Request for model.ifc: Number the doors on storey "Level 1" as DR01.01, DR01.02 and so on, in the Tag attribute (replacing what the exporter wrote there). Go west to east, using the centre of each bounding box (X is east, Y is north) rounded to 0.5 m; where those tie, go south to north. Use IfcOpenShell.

First a look at what the model holds.

```python
import ifcopenshell
import ifcopenshell.util.element
import ifcopenshell.util.placement

model = ifcopenshell.open("model.ifc")
print(model.schema)
storey = next(s for s in model.by_type("IfcBuildingStorey") if s.Name == "Level 1")
doors = [e for e in ifcopenshell.util.element.get_decomposition(storey) if e.is_a("IfcDoor")]
for e in sorted(doors, key=lambda e: e.id()):
    origin = ifcopenshell.util.placement.get_local_placement(e.ObjectPlacement)[:3, 3]
    print(e.id(), e.Tag, e.Name, origin.round(2) + 0.0, sep=" | ")
```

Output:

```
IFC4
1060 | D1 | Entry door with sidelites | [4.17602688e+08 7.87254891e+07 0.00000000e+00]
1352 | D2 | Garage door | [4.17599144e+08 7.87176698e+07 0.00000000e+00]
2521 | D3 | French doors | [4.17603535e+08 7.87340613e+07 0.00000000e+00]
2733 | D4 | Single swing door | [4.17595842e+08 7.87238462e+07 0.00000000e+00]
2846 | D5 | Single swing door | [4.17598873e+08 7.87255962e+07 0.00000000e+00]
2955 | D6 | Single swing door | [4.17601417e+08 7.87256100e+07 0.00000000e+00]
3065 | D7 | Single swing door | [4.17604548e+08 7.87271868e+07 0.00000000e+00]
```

```python
import ifcopenshell
import ifcopenshell.geom
import ifcopenshell.util.element
import ifcopenshell.util.shape

model = ifcopenshell.open("model.ifc")
settings = ifcopenshell.geom.settings()
settings.set("use-world-coords", True)


def centre(element):
    shape = ifcopenshell.geom.create_shape(settings, element)
    return ifcopenshell.util.shape.get_bbox_centroid(shape.geometry)


storey = next(s for s in model.by_type("IfcBuildingStorey") if s.Name == "Level 1")
doors = [e for e in ifcopenshell.util.element.get_decomposition(storey) if e.is_a("IfcDoor")]

# Insertion points can sit at a corner or the storey origin, so sort by the geometry (in metres).
centres = {e: centre(e) for e in doors}
doors.sort(key=lambda e: (round(centres[e][0] / 0.5), centres[e][1]))

for i, e in enumerate(doors, start=1):
    number = f"DR01.{i:02d}"
    e.Tag = number
    print(e.id(), number)

model.write("model-out.ifc")
```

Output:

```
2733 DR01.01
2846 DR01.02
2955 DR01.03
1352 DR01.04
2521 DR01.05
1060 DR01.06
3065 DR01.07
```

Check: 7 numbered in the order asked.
